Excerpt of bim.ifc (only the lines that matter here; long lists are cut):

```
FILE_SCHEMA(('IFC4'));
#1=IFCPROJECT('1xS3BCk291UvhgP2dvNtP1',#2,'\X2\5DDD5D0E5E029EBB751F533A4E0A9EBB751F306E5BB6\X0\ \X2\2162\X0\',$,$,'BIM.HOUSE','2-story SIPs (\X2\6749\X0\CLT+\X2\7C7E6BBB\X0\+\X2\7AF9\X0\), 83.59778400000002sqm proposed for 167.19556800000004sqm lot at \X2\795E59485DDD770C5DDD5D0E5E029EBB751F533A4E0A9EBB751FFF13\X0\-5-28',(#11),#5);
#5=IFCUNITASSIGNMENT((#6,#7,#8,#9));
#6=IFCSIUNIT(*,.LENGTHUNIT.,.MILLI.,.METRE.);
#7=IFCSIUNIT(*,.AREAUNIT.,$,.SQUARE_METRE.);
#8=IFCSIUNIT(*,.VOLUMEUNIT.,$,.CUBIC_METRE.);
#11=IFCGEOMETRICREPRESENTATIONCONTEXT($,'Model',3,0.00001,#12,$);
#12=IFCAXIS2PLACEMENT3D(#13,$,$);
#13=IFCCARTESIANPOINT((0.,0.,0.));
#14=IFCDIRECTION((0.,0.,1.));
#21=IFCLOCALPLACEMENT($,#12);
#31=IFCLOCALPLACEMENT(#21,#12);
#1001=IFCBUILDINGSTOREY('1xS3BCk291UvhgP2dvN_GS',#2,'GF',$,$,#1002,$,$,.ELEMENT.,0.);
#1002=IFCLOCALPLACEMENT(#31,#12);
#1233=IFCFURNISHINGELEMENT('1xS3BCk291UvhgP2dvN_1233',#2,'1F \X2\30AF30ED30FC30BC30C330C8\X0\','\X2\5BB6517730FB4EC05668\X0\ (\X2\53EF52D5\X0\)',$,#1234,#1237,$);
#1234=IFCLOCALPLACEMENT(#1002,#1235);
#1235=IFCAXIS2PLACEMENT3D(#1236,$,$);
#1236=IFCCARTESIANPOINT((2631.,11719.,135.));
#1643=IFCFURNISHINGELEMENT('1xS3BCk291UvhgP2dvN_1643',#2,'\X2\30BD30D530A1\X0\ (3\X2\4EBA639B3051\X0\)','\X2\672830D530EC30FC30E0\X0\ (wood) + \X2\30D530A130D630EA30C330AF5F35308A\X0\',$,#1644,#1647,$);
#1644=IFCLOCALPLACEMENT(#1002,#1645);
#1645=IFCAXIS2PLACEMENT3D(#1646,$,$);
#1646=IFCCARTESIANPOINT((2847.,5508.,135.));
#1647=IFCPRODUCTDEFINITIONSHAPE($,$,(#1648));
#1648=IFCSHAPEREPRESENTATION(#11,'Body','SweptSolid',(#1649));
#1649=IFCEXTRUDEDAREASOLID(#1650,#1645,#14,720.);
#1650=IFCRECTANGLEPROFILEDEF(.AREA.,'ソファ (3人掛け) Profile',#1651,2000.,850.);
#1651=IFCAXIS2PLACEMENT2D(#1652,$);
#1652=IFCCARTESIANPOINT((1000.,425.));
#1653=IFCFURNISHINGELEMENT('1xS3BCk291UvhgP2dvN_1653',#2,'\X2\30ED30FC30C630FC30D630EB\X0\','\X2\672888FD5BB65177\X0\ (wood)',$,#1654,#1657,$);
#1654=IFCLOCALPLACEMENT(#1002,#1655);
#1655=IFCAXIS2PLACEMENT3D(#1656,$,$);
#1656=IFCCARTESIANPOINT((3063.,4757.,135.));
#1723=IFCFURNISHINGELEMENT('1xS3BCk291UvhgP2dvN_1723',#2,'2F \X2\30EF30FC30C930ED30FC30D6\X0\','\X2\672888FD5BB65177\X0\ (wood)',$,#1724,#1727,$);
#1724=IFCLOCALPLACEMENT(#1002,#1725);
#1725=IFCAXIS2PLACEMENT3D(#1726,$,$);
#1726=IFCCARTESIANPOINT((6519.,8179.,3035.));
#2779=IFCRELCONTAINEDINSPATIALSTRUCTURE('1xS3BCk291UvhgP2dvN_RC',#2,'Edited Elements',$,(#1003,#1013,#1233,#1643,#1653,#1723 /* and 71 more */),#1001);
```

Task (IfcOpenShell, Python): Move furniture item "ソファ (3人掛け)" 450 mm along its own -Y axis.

```python
import ifcopenshell
import ifcopenshell.api.geometry
import ifcopenshell.util.placement
import ifcopenshell.util.unit

model = ifcopenshell.open("bim.ifc")
unit_scale = ifcopenshell.util.unit.calculate_unit_scale(model)

item = model.by_guid("1xS3BCk291UvhgP2dvN_1643")
matrix = ifcopenshell.util.placement.get_local_placement(item.ObjectPlacement)
matrix[:3, 3] -= matrix[:3, 1] * 0.45 / unit_scale
ifcopenshell.api.geometry.edit_object_placement(model, product=item, matrix=matrix, is_si=False)

print(ifcopenshell.util.placement.get_local_placement(item.ObjectPlacement).round(3) + 0.0)

model.write("bim_edited.ifc")
```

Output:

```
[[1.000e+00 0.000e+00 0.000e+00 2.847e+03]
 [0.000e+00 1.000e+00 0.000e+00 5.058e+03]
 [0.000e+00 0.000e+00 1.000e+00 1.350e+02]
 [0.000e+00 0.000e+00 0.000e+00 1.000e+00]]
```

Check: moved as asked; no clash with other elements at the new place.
